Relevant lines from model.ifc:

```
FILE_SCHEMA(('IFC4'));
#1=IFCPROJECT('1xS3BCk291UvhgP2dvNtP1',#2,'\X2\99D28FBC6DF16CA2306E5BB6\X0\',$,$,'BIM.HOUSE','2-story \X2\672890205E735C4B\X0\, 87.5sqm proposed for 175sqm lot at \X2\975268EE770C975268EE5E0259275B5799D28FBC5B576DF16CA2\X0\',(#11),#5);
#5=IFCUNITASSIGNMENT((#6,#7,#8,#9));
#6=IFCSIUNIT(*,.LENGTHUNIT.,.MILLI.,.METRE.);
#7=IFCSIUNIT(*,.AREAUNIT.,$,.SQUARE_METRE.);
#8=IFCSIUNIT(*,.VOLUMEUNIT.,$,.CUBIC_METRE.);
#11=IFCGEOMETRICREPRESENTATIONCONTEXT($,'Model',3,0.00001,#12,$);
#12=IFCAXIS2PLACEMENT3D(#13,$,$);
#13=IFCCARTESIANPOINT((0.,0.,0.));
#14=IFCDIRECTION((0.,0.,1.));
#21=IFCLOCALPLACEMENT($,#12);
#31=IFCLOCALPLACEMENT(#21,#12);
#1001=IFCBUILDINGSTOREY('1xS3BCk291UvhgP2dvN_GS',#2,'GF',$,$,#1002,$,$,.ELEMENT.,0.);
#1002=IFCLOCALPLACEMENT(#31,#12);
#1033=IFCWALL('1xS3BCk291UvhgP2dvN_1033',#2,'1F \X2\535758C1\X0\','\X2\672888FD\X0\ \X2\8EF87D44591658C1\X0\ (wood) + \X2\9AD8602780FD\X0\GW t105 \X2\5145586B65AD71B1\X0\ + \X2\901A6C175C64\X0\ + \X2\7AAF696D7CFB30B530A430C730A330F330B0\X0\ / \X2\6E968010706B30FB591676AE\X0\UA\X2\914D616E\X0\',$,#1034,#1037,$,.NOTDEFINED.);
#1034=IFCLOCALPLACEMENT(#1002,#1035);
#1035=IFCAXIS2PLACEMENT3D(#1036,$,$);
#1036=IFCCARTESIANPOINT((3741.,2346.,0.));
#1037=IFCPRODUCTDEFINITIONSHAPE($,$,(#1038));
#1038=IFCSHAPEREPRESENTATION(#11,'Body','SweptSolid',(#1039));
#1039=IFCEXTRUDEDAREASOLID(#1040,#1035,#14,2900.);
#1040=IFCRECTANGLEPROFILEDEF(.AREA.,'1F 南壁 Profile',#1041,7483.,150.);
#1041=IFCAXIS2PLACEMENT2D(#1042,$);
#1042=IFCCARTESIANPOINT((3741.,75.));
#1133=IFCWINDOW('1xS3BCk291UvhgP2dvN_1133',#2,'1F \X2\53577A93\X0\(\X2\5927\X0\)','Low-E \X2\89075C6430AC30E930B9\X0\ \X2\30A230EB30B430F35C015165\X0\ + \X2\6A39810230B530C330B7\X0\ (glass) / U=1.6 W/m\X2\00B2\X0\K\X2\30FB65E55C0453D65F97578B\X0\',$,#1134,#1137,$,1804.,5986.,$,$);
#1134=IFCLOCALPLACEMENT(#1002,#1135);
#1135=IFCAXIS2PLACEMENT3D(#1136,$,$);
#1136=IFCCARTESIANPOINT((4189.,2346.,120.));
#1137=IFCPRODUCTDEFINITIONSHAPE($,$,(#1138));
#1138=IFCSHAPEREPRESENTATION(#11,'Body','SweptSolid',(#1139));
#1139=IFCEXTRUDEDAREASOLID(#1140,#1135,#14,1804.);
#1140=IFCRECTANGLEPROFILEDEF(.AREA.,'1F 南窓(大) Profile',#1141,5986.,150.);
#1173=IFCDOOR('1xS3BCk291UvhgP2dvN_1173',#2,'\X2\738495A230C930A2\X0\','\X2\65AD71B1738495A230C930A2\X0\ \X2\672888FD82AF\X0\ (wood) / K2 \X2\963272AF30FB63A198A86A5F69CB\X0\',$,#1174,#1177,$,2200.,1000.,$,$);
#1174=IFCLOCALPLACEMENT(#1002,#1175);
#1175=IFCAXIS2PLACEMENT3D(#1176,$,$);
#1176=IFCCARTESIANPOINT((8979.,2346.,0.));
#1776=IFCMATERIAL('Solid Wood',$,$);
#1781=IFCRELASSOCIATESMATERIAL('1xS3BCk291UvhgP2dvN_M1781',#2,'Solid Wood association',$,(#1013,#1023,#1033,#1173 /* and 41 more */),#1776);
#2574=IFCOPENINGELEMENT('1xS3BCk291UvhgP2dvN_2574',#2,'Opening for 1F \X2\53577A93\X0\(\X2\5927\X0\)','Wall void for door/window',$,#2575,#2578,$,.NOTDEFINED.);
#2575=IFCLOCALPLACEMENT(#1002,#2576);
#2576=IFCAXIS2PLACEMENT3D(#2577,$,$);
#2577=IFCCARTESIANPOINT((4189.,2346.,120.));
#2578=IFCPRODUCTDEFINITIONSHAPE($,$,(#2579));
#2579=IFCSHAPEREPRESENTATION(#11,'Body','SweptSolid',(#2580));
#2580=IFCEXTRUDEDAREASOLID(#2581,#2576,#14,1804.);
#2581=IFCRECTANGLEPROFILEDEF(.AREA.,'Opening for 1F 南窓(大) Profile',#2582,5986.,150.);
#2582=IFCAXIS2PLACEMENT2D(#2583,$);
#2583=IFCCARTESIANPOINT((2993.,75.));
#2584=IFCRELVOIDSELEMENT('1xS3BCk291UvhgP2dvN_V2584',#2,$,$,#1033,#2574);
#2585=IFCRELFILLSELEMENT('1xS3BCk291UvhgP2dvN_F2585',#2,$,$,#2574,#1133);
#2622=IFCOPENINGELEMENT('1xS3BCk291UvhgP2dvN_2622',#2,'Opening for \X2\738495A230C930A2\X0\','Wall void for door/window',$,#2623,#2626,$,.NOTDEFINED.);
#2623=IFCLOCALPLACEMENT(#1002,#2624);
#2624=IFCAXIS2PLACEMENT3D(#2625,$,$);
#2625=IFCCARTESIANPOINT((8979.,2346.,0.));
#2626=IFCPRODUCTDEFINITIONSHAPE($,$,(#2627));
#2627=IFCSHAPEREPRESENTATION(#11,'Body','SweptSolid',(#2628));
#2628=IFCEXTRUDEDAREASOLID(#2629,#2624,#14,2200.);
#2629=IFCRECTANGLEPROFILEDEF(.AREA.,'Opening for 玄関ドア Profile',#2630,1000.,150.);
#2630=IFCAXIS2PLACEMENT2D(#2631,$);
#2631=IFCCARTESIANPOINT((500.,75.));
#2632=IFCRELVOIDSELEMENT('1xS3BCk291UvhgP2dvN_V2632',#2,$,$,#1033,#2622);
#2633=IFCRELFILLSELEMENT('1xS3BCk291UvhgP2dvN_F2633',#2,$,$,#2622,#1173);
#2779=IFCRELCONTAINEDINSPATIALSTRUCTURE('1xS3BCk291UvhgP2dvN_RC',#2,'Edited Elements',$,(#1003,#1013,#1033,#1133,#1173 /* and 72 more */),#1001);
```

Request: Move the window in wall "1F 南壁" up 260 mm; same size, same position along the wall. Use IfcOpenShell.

```python
import numpy as np
import ifcopenshell
import ifcopenshell.api.geometry
import ifcopenshell.util.placement
import ifcopenshell.util.unit

model = ifcopenshell.open("model.ifc")
unit_scale = ifcopenshell.util.unit.calculate_unit_scale(model)

window = model.by_guid("1xS3BCk291UvhgP2dvN_1133")
opening = window.FillsVoids[0].RelatingOpeningElement
dz = 0.26 / unit_scale

shift = np.array([0.0, 0.0, dz])
# The window is not placed relative to its opening, so move both.
for product in (opening, window):
    matrix = ifcopenshell.util.placement.get_local_placement(product.ObjectPlacement)
    matrix[:3, 3] += shift
    ifcopenshell.api.geometry.edit_object_placement(model, product=product, matrix=matrix, is_si=False)

print(f"moved by {dz * unit_scale:+.3f} m")

model.write("model_edited.ifc")
```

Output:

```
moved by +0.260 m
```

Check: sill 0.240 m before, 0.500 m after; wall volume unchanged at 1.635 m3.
